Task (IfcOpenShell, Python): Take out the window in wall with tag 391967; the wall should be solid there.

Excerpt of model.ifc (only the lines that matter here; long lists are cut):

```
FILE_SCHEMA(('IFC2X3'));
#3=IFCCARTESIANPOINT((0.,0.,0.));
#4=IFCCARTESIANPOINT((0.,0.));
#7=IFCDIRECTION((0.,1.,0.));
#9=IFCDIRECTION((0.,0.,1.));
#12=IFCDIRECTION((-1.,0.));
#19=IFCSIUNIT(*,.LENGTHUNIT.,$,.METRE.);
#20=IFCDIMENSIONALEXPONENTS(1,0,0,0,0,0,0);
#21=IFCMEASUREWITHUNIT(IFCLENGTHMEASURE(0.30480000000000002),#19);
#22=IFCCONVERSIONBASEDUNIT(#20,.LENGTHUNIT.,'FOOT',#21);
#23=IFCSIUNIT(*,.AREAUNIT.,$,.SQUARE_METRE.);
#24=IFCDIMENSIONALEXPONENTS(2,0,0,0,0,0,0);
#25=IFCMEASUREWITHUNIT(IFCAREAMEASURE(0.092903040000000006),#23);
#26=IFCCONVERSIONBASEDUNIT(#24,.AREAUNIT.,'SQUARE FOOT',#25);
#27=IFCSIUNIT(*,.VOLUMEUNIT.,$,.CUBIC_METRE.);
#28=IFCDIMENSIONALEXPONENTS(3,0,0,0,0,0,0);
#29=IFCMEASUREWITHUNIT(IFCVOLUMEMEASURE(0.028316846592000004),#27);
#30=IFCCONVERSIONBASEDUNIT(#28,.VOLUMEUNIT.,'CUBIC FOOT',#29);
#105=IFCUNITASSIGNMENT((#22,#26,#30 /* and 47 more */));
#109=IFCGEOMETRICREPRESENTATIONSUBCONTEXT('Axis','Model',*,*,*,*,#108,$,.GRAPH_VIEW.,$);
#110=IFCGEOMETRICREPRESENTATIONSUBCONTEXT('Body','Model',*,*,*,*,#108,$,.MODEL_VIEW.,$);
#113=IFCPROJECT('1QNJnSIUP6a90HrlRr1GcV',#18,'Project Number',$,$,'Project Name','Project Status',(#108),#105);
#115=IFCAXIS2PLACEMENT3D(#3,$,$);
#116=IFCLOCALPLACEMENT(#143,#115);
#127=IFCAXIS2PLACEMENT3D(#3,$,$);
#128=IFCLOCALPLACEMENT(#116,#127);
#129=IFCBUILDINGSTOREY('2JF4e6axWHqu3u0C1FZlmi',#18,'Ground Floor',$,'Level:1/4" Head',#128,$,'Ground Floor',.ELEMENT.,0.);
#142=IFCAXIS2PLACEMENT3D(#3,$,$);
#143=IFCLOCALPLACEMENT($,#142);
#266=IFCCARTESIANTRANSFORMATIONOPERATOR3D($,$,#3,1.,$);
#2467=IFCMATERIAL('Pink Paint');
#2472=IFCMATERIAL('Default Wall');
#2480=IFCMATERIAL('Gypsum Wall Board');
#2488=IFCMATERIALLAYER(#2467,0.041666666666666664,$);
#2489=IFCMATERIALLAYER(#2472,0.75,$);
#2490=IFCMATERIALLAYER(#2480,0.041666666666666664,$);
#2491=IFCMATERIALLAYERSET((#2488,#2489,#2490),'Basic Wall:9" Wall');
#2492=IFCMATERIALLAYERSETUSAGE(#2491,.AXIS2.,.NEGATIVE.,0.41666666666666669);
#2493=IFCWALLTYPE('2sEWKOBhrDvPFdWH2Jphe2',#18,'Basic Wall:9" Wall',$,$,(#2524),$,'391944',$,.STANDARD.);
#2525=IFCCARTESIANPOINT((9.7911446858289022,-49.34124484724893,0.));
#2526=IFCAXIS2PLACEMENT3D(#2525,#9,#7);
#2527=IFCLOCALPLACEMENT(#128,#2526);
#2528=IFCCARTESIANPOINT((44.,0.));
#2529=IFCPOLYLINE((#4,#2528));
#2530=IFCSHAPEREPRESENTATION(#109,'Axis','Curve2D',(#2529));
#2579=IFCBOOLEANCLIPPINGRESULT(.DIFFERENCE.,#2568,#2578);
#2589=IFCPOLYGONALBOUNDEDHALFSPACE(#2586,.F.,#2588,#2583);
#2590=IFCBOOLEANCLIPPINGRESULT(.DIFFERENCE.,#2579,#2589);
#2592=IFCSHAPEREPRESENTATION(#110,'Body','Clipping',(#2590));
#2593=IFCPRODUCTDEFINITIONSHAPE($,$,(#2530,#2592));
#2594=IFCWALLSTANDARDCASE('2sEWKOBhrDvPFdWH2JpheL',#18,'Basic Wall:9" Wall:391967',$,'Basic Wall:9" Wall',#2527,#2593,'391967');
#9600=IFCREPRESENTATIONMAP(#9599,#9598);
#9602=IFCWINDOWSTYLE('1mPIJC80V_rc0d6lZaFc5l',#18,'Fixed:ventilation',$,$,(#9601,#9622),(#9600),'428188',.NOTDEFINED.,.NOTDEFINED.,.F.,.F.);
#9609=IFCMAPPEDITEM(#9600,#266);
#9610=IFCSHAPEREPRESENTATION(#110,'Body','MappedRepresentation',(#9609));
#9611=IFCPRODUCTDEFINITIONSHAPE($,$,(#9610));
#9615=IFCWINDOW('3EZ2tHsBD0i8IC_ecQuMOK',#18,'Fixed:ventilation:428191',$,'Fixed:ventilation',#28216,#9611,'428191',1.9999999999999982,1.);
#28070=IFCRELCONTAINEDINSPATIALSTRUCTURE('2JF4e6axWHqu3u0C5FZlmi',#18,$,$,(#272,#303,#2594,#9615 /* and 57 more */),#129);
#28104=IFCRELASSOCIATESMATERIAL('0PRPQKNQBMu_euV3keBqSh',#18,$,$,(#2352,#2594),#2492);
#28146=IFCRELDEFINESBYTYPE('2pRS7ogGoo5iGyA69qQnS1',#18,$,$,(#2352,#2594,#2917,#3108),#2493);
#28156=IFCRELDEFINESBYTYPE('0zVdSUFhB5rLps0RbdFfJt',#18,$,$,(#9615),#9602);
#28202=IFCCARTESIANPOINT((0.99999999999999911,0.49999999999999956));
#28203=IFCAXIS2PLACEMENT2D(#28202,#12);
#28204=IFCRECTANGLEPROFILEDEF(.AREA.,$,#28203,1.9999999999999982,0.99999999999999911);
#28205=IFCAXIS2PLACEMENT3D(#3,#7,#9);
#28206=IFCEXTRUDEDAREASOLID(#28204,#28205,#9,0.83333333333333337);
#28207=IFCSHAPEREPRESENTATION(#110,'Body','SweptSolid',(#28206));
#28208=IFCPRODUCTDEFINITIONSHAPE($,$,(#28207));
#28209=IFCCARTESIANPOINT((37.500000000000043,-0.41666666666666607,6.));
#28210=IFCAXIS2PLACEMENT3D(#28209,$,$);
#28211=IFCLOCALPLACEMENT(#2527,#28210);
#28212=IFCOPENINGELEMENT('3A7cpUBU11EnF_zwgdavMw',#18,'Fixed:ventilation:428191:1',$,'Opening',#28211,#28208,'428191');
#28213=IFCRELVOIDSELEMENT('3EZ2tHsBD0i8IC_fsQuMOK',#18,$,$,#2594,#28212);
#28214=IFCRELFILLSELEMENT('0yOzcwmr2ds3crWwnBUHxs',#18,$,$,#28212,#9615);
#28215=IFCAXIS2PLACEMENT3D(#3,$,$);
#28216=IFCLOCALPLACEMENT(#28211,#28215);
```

```python
import ifcopenshell
import ifcopenshell.api.feature
import ifcopenshell.api.root
import ifcopenshell.geom
import ifcopenshell.util.shape

model = ifcopenshell.open("model.ifc")
settings = ifcopenshell.geom.settings()


def volume(element):
    """Net volume in cubic metres, openings subtracted."""
    shape = ifcopenshell.geom.create_shape(settings, element)
    return ifcopenshell.util.shape.get_volume(shape.geometry)


window = model.by_id(9615)
opening = window.FillsVoids[0].RelatingOpeningElement
wall = opening.VoidsElements[0].RelatingBuildingElement
before = volume(wall)

ifcopenshell.api.root.remove_product(model, product=window)
ifcopenshell.api.feature.remove_feature(model, feature=opening)

after = volume(wall)

print(f"wall volume {before:.3f} -> {after:.3f} m3")

model.write("model_edited.ifc")
```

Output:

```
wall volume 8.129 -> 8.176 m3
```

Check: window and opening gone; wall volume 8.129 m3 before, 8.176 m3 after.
